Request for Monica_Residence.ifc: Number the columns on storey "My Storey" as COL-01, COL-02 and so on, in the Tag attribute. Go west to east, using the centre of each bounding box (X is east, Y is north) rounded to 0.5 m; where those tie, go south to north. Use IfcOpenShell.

First a look at what the model holds.

```python
import ifcopenshell
import ifcopenshell.util.element
import ifcopenshell.util.placement

model = ifcopenshell.open("Monica_Residence.ifc")
print(model.schema)
storey = next(s for s in model.by_type("IfcBuildingStorey") if s.Name == "My Storey")
columns = [e for e in ifcopenshell.util.element.get_decomposition(storey) if e.is_a("IfcColumn")]
for e in sorted(columns, key=lambda e: e.id()):
    origin = ifcopenshell.util.placement.get_local_placement(e.ObjectPlacement)[:3, 3]
    print(e.id(), e.Tag, e.Name, origin.round(2) + 0.0, sep=" | ")
```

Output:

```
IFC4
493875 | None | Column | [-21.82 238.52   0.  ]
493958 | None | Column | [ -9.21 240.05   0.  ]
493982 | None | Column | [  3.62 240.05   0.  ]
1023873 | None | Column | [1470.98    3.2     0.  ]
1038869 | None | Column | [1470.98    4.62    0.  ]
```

```python
import ifcopenshell
import ifcopenshell.geom
import ifcopenshell.util.element
import ifcopenshell.util.shape

model = ifcopenshell.open("Monica_Residence.ifc")
settings = ifcopenshell.geom.settings()
settings.set("use-world-coords", True)


def centre(element):
    shape = ifcopenshell.geom.create_shape(settings, element)
    return ifcopenshell.util.shape.get_bbox_centroid(shape.geometry)


storey = next(s for s in model.by_type("IfcBuildingStorey") if s.Name == "My Storey")
columns = [e for e in ifcopenshell.util.element.get_decomposition(storey) if e.is_a("IfcColumn")]

# Insertion points can sit at a corner or the storey origin, so sort by the geometry (in metres).
centres = {e: centre(e) for e in columns}
columns.sort(key=lambda e: (round(centres[e][0] / 0.5), centres[e][1]))

for i, e in enumerate(columns, start=1):
    number = f"COL-{i:02d}"
    e.Tag = number
    print(e.id(), number)

model.write("Monica_Residence_edited.ifc")
```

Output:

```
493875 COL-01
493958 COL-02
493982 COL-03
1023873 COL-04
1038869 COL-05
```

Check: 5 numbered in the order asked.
